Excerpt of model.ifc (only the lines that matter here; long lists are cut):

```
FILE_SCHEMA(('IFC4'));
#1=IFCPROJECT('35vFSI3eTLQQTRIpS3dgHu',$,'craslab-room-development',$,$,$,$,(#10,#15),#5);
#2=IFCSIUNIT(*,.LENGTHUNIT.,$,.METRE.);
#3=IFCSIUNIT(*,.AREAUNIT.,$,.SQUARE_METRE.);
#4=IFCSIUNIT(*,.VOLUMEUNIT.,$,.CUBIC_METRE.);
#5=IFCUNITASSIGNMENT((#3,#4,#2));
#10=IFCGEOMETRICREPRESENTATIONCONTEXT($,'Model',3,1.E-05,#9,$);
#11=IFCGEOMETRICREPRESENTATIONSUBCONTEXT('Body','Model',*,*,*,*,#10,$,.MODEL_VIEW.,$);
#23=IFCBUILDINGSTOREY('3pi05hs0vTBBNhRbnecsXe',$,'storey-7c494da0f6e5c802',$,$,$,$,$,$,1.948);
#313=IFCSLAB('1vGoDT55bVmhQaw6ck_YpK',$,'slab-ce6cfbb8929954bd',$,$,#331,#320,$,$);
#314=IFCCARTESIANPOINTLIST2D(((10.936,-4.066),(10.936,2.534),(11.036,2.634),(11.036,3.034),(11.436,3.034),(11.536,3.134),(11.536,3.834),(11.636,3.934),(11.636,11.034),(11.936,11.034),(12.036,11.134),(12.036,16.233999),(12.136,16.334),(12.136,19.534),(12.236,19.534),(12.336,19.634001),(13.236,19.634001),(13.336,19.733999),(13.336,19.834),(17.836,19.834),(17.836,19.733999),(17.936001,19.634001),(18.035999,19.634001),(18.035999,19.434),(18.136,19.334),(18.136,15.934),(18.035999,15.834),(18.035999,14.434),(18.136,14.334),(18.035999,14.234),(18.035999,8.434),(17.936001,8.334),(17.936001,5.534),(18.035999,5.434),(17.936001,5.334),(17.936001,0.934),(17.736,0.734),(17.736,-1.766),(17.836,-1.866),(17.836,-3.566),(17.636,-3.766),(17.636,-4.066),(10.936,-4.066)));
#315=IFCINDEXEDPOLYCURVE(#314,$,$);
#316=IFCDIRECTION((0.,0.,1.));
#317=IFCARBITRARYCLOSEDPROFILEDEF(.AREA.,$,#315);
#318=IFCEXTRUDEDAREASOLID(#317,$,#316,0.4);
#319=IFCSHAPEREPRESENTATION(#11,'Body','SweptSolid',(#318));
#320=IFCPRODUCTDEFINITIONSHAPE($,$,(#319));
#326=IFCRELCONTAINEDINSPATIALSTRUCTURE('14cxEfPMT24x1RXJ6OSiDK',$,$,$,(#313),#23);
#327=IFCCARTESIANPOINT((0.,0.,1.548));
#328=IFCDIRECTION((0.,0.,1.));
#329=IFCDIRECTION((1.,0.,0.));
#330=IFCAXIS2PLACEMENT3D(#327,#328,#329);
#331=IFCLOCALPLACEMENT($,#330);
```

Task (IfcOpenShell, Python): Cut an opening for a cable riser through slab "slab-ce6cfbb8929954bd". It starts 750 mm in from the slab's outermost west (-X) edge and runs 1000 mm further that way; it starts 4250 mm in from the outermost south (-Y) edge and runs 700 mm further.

```python
import numpy as np
import ifcopenshell
import ifcopenshell.api.feature
import ifcopenshell.api.geometry
import ifcopenshell.api.root
import ifcopenshell.geom
import ifcopenshell.util.placement
import ifcopenshell.util.representation
import ifcopenshell.util.shape
import ifcopenshell.util.unit

model = ifcopenshell.open("model.ifc")
unit_scale = ifcopenshell.util.unit.calculate_unit_scale(model)
settings = ifcopenshell.geom.settings()


def volume(element):
    """Net volume in cubic metres, openings subtracted."""
    shape = ifcopenshell.geom.create_shape(settings, element)
    return ifcopenshell.util.shape.get_volume(shape.geometry)


slab = model.by_guid("1vGoDT55bVmhQaw6ck_YpK")
before = volume(slab)

# Extent in the slab's own axes, in metres. The edges named are its -X and -Y sides.
slab_shape = ifcopenshell.geom.create_shape(settings, slab)
vertices = ifcopenshell.util.shape.get_vertices(slab_shape.geometry)
x_min, y_min, bottom = vertices.min(axis=0)
top = vertices[:, 2].max()

opening = ifcopenshell.api.root.create_entity(model, ifc_class="IfcOpeningElement", name="Cable riser opening", predefined_type="OPENING")
context = ifcopenshell.util.representation.get_context(model, "Model", "Body", "MODEL_VIEW")
width, depth = 1, 0.7
outline = [(0.0, 0.0), (width, 0.0), (width, depth), (0.0, depth), (0.0, 0.0)]
# Overshoot both faces by 50 mm so the cut is clean.
shape = ifcopenshell.api.geometry.add_slab_representation(
    model, context=context, depth=top - bottom + 0.1, polyline=outline
)
ifcopenshell.api.geometry.assign_representation(model, product=opening, representation=shape)

matrix = ifcopenshell.util.placement.get_local_placement(slab.ObjectPlacement)
matrix[:, 3] = matrix @ np.append(np.array([x_min + 0.75, y_min + 4.25, bottom - 0.05]) / unit_scale, 1.0)
ifcopenshell.api.geometry.edit_object_placement(model, product=opening, matrix=matrix, is_si=False)
ifcopenshell.api.feature.add_feature(model, feature=opening, element=slab)

after = volume(slab)

print(f"slab volume {before:.3f} -> {after:.3f} m3")

model.write("model_updated.ifc")
```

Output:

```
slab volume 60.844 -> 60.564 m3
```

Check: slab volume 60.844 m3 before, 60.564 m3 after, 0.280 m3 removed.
